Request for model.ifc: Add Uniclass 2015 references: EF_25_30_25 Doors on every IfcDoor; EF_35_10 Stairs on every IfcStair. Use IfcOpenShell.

First a look at what the model holds.

```python
import ifcopenshell

model = ifcopenshell.open("model.ifc")
print(model.schema)
print("classifications:", [c.Name for c in model.by_type("IfcClassification")])
for ifc_class in ("IfcDoor", "IfcRoof", "IfcStair", "IfcWall", "IfcWindow"):
    print(ifc_class, len(model.by_type(ifc_class)))
```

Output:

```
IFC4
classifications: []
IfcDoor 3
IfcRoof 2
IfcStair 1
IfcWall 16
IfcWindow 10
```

```python
import ifcopenshell
import ifcopenshell.api.classification

model = ifcopenshell.open("model.ifc")

system = ifcopenshell.api.classification.add_classification(model, classification="Uniclass 2015")

codes = {
    "IfcDoor": ("EF_25_30_25", "Doors"),
    "IfcStair": ("EF_35_10", "Stairs"),
}
for ifc_class, (code, name) in codes.items():
    products = model.by_type(ifc_class)
    ifcopenshell.api.classification.add_reference(
        model, products=products, classification=system, identification=code, name=name
    )
    print(code, len(products))

model.write("model-out.ifc")
```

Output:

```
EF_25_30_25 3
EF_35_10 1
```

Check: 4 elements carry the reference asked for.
